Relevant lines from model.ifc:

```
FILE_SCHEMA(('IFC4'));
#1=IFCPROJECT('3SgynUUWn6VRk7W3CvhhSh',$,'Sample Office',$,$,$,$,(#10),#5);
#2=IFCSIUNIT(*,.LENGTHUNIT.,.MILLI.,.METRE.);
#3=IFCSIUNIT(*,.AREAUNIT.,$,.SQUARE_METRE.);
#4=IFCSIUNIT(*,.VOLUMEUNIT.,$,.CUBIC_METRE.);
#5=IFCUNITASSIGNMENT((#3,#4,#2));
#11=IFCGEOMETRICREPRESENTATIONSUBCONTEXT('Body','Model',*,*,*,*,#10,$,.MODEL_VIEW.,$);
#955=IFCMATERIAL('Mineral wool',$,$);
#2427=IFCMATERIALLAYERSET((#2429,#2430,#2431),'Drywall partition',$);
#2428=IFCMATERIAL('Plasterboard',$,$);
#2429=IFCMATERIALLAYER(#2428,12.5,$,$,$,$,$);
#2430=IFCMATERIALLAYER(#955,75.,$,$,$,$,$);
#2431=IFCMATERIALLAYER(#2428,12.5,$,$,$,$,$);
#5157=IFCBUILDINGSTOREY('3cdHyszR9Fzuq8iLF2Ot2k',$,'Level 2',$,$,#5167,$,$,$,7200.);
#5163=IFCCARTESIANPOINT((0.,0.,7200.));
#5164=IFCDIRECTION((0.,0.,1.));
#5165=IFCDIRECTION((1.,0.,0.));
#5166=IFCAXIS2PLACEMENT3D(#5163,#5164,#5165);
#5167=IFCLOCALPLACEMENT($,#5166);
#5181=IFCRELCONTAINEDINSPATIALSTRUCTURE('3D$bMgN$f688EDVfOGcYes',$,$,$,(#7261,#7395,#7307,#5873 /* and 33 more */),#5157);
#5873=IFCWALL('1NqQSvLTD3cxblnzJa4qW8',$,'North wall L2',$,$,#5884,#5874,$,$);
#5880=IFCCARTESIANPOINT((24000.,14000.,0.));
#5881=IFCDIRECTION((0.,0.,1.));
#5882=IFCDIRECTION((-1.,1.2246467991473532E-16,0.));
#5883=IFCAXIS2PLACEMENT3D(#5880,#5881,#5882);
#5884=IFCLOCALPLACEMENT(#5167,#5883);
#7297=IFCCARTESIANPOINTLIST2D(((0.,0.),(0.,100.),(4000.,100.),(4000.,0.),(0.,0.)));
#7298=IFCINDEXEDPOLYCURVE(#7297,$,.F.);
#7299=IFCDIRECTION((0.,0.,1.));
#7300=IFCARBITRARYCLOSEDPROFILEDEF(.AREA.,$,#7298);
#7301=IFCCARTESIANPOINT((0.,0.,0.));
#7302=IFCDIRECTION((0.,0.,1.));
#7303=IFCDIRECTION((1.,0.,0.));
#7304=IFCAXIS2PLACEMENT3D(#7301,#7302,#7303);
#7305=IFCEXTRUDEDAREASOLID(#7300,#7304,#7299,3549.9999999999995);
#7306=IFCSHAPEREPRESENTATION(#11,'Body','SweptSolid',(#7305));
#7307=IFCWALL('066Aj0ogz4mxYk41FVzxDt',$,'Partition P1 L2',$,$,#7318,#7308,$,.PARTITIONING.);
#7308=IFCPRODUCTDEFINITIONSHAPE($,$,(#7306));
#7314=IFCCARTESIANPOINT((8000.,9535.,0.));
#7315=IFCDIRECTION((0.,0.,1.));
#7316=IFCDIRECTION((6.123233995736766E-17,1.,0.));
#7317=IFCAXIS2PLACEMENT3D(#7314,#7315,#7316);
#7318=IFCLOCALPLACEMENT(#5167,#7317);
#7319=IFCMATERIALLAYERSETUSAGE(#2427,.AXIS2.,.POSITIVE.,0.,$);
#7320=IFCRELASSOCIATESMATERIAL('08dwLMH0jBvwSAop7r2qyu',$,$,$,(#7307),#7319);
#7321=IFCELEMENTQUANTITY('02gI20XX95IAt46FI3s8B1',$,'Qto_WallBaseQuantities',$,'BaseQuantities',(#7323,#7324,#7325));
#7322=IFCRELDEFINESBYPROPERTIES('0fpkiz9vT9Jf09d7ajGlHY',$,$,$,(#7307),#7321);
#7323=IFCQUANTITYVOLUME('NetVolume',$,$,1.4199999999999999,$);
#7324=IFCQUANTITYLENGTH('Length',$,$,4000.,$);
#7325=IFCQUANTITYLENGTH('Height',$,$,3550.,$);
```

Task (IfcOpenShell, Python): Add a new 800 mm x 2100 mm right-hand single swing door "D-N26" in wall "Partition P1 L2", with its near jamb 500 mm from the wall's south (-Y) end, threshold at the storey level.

```python
import numpy as np
import ifcopenshell
import ifcopenshell.api.feature
import ifcopenshell.api.geometry
import ifcopenshell.api.pset
import ifcopenshell.api.root
import ifcopenshell.api.spatial
import ifcopenshell.geom
import ifcopenshell.util.element
import ifcopenshell.util.placement
import ifcopenshell.util.representation
import ifcopenshell.util.shape
import ifcopenshell.util.unit

model = ifcopenshell.open("model.ifc")
unit_scale = ifcopenshell.util.unit.calculate_unit_scale(model)
volume_scale = ifcopenshell.util.unit.calculate_unit_scale(model, "VOLUMEUNIT")
settings = ifcopenshell.geom.settings()


def volume(element):
    """Net volume in cubic metres, openings subtracted."""
    shape = ifcopenshell.geom.create_shape(settings, element)
    return ifcopenshell.util.shape.get_volume(shape.geometry)


wall = model.by_guid("066Aj0ogz4mxYk41FVzxDt")
storey = ifcopenshell.util.element.get_container(wall, ifc_class="IfcBuildingStorey")
context = ifcopenshell.util.representation.get_context(model, "Model", "Body", "MODEL_VIEW")
before = volume(wall)

width, height, from_end, sill = 0.8, 2.1, 0.5, 0.0  # metres

# The wall runs along its own X axis, and the end named is its -X end.
wall_shape = ifcopenshell.geom.create_shape(settings, wall)
x, y, z = ifcopenshell.util.shape.get_vertices(wall_shape.geometry).T
start = x.min() + from_end
face, thickness = float(y.min()), float(y.max() - y.min())
wall_matrix = ifcopenshell.util.placement.get_local_placement(wall.ObjectPlacement)
level = ifcopenshell.util.placement.get_local_placement(storey.ObjectPlacement)[2, 3]


def in_wall(x, y):
    """Placement at x, y metres in the wall's axes, at sill height."""
    matrix = wall_matrix.copy()
    matrix[:, 3] = wall_matrix @ np.array([x / unit_scale, y / unit_scale, 0.0, 1.0])
    matrix[2, 3] = level + sill / unit_scale
    return matrix


# Opening: a box that overshoots both wall faces by 50 mm.
opening = ifcopenshell.api.root.create_entity(model, ifc_class="IfcOpeningElement", predefined_type="OPENING")
box = ifcopenshell.api.geometry.add_wall_representation(
    model, context=context, length=width, height=height, thickness=thickness + 0.1
)
ifcopenshell.api.geometry.assign_representation(model, product=opening, representation=box)
ifcopenshell.api.geometry.edit_object_placement(model, product=opening, matrix=in_wall(start, face - 0.05), is_si=False)
ifcopenshell.api.feature.add_feature(model, feature=opening, element=wall)

door = ifcopenshell.api.root.create_entity(model, ifc_class="IfcDoor", name="D-N26", predefined_type="DOOR")
door.OverallWidth, door.OverallHeight = width / unit_scale, height / unit_scale
door.OperationType = "SINGLE_SWING_RIGHT"
body = ifcopenshell.api.geometry.add_door_representation(
    model,
    context=context,
    overall_width=door.OverallWidth,
    overall_height=door.OverallHeight,
    operation_type="SINGLE_SWING_RIGHT",
    lining_properties={"LiningDepth": thickness / unit_scale, "ThresholdDepth": thickness / unit_scale},
)
ifcopenshell.api.geometry.assign_representation(model, product=door, representation=body)
ifcopenshell.api.spatial.assign_container(model, products=[door], relating_structure=storey)
ifcopenshell.api.feature.add_filling(model, opening=opening, element=door)

# The lining spans the wall, so the door starts at the wall face.
ifcopenshell.api.geometry.edit_object_placement(model, product=door, matrix=in_wall(start, face), is_si=False)

after = volume(wall)

# Update the wall's stored quantities.
qto = model.by_id(ifcopenshell.util.element.get_pset(wall, "Qto_WallBaseQuantities", should_inherit=False)["id"])
ifcopenshell.api.pset.edit_qto(model, qto=qto, properties={"NetVolume": after / volume_scale})

print(f"wall volume {before:.3f} -> {after:.3f} m3")

model.write("model_edited.ifc")
```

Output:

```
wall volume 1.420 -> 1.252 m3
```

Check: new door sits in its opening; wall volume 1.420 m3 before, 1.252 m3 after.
